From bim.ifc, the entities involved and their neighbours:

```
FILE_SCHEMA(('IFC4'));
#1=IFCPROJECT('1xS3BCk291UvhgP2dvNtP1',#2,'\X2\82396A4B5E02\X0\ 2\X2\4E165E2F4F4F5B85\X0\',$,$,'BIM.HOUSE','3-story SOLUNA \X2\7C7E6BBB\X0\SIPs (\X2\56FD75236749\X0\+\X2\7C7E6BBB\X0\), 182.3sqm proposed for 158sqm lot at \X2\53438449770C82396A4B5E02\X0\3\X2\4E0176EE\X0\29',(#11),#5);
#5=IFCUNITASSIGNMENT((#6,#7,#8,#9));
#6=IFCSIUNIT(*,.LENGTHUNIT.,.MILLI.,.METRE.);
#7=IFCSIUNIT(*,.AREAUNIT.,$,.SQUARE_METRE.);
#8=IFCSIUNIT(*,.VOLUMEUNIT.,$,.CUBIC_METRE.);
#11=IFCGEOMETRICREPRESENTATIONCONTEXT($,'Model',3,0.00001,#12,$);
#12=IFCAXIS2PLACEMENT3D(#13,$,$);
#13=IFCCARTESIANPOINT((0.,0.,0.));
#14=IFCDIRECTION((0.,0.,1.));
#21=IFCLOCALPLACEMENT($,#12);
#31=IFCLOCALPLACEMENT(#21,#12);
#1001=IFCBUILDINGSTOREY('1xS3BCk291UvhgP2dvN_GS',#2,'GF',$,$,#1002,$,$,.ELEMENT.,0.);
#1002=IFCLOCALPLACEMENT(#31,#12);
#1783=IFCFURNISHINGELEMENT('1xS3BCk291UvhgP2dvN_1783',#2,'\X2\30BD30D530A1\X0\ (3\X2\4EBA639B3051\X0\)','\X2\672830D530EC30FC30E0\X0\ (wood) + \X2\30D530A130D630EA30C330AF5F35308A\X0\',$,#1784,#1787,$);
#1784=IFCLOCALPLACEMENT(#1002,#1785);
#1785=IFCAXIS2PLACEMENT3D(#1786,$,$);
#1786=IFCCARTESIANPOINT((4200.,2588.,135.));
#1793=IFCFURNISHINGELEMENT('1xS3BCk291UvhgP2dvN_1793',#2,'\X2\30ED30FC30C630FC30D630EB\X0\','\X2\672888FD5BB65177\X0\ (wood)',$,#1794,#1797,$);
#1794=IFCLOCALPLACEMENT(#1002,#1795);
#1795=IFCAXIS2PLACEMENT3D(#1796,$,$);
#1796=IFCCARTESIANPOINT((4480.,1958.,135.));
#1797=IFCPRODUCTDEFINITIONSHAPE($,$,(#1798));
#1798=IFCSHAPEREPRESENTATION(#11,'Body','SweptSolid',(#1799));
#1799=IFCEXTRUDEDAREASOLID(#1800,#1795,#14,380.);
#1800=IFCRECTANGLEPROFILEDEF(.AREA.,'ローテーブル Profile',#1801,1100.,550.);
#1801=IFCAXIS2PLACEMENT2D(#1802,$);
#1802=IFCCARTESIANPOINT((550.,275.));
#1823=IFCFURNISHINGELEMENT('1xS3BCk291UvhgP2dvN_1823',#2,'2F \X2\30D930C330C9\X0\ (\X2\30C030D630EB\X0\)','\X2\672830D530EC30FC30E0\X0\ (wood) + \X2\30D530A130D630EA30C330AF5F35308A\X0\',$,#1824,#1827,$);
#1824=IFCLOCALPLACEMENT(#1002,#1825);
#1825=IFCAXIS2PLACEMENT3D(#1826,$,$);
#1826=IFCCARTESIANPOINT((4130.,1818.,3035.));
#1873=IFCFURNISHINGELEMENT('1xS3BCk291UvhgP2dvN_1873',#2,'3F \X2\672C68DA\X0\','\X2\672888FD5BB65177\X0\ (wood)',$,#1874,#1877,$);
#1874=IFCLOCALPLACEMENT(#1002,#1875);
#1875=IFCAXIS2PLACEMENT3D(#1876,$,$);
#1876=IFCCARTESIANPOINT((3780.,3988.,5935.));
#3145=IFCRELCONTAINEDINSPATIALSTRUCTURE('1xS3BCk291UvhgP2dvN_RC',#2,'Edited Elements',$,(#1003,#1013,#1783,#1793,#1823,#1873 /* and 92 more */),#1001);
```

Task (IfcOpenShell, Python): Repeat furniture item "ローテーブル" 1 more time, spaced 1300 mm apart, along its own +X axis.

```python
import ifcopenshell
import ifcopenshell.api.geometry
import ifcopenshell.api.root
import ifcopenshell.util.element
import ifcopenshell.util.placement
import ifcopenshell.util.unit

model = ifcopenshell.open("bim.ifc")
unit_scale = ifcopenshell.util.unit.calculate_unit_scale(model)


def reuse_history(source, copy):
    """copy_class also copies each property set's owner history, people and application; keep the originals."""
    for rel in copy.IsDefinedBy:
        if rel.is_a("IfcRelDefinesByProperties") and (history := rel.RelatingPropertyDefinition.OwnerHistory):
            rel.RelatingPropertyDefinition.OwnerHistory = source.OwnerHistory
            ifcopenshell.util.element.remove_deep2(model, history)


source = model.by_id(1793)
base = ifcopenshell.util.placement.get_local_placement(source.ObjectPlacement)
step = base[:3, 0] * 1.3 / unit_scale

for i in range(1, 2):
    copy = ifcopenshell.api.root.copy_class(model, product=source)
    copy.Representation = ifcopenshell.util.element.copy_deep(
        model, source.Representation, exclude=["IfcGeometricRepresentationContext", "IfcRepresentationMap"]
    )
    reuse_history(source, copy)
    matrix = base.copy()
    matrix[:3, 3] += i * step
    print("added at", matrix[:3, 3].round(3) + 0.0)
    ifcopenshell.api.geometry.edit_object_placement(model, product=copy, matrix=matrix, is_si=False)

model.write("bim_v2.ifc")
```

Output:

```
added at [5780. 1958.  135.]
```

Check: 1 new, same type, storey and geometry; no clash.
